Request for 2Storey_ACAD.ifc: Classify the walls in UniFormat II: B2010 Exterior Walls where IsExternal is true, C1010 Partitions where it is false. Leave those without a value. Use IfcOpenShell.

First a look at what the model holds.

```python
import ifcopenshell
import ifcopenshell.util.element

model = ifcopenshell.open("2Storey_ACAD.ifc")
print(model.schema)
print("classifications:", [c.Name for c in model.by_type("IfcClassification")])
values = [ifcopenshell.util.element.get_pset(e, "Pset_WallCommon", "IsExternal") for e in model.by_type("IfcWall")]
for value in (True, False, None):
    print("IsExternal", value, values.count(value))
```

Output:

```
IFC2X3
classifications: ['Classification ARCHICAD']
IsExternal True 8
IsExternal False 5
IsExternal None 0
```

```python
import ifcopenshell
import ifcopenshell.api.classification
import ifcopenshell.util.element

model = ifcopenshell.open("2Storey_ACAD.ifc")

# IFC2X3 requires Source and Edition and has no link from the project to the system.
system = model.create_entity("IfcClassification", Source="ASTM", Edition="E1557", Name="UniFormat II")

walls = model.by_type("IfcWall")
external = {e: ifcopenshell.util.element.get_pset(e, "Pset_WallCommon", "IsExternal") for e in walls}
for flag, code, name in ((True, "B2010", "Exterior Walls"), (False, "C1010", "Partitions")):
    products = [e for e in walls if external[e] is flag]
    ifcopenshell.api.classification.add_reference(
        model, products=products, classification=system, identification=code, name=name
    )
    print(code, len(products))

model.write("2Storey_ACAD_rev.ifc")
```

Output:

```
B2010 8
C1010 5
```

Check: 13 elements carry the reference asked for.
